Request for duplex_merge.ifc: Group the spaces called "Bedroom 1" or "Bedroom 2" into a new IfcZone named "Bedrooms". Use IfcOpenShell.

First a look at what the model holds.

```python
import ifcopenshell

model = ifcopenshell.open("duplex_merge.ifc")
print(model.schema)
seen = {}
for space in model.by_type("IfcSpace"):
    seen[space.LongName] = seen.get(space.LongName, 0) + 1
for name, count in sorted(seen.items(), key=str):
    print(count, "x", name)
print("zones:", [z.Name for z in model.by_type("IfcZone")][:20])
```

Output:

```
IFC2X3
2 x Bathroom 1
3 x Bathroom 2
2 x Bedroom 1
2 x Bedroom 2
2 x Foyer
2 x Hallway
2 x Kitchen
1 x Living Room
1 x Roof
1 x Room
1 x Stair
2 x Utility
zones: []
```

```python
import ifcopenshell
import ifcopenshell.api.group
import ifcopenshell.api.root

model = ifcopenshell.open("duplex_merge.ifc")

names = {"Bedroom 1", "Bedroom 2"}
spaces = [s for s in model.by_type("IfcSpace") if s.LongName in names]

zone = ifcopenshell.api.root.create_entity(model, ifc_class="IfcZone", name="Bedrooms")
ifcopenshell.api.group.assign_group(model, products=spaces, group=zone)
print(len(spaces), "spaces in", zone.Name)

model.write("duplex_merge-out.ifc")
```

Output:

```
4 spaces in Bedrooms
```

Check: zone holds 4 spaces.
